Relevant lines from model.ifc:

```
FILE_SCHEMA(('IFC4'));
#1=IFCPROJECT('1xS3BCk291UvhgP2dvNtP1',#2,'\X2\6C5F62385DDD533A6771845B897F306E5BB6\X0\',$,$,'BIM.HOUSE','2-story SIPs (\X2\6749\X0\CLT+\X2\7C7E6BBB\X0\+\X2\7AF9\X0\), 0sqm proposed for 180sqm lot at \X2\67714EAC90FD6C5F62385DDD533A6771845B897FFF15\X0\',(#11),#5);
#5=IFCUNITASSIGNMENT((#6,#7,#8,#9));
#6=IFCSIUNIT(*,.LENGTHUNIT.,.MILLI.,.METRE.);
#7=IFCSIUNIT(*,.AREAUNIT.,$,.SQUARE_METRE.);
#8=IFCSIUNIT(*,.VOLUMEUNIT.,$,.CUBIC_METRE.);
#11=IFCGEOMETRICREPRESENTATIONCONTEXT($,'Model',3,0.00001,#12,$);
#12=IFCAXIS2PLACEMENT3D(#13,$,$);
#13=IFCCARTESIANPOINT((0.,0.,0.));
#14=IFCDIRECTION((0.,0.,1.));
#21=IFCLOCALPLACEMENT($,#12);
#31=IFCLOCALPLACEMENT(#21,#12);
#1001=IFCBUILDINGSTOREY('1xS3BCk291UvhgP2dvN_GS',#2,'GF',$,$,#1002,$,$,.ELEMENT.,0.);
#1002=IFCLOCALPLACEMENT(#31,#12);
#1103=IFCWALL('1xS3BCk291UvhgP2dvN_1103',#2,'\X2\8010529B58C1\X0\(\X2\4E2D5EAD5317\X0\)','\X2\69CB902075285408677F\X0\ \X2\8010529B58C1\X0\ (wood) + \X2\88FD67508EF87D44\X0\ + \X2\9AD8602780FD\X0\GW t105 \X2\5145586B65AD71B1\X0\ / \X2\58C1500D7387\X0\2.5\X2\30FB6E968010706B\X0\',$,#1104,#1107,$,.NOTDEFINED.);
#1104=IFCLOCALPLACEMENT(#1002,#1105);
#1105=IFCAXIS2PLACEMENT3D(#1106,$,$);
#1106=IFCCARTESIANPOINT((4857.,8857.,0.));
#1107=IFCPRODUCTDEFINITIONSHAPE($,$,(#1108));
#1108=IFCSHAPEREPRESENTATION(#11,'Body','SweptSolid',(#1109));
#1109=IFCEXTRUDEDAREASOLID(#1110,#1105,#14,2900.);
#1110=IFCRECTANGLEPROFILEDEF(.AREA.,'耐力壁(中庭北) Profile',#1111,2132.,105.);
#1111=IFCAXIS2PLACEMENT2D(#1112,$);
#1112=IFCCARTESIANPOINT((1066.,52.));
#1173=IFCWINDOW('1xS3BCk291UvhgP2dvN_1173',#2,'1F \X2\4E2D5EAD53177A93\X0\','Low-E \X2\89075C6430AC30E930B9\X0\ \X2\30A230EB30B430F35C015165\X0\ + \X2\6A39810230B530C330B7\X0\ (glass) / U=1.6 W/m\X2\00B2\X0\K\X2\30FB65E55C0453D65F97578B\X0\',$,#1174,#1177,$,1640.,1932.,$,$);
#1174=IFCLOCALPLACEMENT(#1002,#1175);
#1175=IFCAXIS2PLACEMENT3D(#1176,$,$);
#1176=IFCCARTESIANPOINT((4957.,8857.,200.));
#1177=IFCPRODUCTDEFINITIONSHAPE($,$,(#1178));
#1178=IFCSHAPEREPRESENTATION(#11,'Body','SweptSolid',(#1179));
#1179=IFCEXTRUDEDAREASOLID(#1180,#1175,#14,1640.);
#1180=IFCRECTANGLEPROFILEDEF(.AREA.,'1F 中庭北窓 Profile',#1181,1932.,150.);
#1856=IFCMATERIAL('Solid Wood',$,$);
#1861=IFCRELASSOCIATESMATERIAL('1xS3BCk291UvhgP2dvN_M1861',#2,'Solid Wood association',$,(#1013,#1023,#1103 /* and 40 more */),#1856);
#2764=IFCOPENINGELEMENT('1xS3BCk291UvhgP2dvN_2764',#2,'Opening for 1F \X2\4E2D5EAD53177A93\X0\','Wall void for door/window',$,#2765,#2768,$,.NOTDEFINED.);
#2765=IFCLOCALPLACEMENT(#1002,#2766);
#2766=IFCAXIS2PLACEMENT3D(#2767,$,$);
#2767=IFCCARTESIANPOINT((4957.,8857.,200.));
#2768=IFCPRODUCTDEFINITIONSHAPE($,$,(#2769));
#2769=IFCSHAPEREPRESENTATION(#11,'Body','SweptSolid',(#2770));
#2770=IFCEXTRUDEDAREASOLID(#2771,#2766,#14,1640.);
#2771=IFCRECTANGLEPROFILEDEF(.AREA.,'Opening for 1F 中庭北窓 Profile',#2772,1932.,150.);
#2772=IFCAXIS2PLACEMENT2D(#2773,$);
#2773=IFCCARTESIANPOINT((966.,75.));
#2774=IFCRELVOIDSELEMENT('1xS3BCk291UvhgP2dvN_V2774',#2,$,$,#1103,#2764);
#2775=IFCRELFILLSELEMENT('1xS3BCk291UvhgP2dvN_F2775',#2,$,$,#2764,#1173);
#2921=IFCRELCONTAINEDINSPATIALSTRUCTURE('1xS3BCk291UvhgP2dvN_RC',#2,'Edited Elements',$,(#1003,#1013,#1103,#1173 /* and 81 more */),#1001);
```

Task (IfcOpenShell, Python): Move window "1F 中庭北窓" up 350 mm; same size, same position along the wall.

```python
import numpy as np
import ifcopenshell
import ifcopenshell.api.geometry
import ifcopenshell.util.placement
import ifcopenshell.util.unit

model = ifcopenshell.open("model.ifc")
unit_scale = ifcopenshell.util.unit.calculate_unit_scale(model)

window = model.by_id(1173)
opening = window.FillsVoids[0].RelatingOpeningElement
dz = 0.35 / unit_scale

shift = np.array([0.0, 0.0, dz])
# The window is not placed relative to its opening, so move both.
for product in (opening, window):
    matrix = ifcopenshell.util.placement.get_local_placement(product.ObjectPlacement)
    matrix[:3, 3] += shift
    ifcopenshell.api.geometry.edit_object_placement(model, product=product, matrix=matrix, is_si=False)

print(f"moved by {dz * unit_scale:+.3f} m")

model.write("model-out.ifc")
```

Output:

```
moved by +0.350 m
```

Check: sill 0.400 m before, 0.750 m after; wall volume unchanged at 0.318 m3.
